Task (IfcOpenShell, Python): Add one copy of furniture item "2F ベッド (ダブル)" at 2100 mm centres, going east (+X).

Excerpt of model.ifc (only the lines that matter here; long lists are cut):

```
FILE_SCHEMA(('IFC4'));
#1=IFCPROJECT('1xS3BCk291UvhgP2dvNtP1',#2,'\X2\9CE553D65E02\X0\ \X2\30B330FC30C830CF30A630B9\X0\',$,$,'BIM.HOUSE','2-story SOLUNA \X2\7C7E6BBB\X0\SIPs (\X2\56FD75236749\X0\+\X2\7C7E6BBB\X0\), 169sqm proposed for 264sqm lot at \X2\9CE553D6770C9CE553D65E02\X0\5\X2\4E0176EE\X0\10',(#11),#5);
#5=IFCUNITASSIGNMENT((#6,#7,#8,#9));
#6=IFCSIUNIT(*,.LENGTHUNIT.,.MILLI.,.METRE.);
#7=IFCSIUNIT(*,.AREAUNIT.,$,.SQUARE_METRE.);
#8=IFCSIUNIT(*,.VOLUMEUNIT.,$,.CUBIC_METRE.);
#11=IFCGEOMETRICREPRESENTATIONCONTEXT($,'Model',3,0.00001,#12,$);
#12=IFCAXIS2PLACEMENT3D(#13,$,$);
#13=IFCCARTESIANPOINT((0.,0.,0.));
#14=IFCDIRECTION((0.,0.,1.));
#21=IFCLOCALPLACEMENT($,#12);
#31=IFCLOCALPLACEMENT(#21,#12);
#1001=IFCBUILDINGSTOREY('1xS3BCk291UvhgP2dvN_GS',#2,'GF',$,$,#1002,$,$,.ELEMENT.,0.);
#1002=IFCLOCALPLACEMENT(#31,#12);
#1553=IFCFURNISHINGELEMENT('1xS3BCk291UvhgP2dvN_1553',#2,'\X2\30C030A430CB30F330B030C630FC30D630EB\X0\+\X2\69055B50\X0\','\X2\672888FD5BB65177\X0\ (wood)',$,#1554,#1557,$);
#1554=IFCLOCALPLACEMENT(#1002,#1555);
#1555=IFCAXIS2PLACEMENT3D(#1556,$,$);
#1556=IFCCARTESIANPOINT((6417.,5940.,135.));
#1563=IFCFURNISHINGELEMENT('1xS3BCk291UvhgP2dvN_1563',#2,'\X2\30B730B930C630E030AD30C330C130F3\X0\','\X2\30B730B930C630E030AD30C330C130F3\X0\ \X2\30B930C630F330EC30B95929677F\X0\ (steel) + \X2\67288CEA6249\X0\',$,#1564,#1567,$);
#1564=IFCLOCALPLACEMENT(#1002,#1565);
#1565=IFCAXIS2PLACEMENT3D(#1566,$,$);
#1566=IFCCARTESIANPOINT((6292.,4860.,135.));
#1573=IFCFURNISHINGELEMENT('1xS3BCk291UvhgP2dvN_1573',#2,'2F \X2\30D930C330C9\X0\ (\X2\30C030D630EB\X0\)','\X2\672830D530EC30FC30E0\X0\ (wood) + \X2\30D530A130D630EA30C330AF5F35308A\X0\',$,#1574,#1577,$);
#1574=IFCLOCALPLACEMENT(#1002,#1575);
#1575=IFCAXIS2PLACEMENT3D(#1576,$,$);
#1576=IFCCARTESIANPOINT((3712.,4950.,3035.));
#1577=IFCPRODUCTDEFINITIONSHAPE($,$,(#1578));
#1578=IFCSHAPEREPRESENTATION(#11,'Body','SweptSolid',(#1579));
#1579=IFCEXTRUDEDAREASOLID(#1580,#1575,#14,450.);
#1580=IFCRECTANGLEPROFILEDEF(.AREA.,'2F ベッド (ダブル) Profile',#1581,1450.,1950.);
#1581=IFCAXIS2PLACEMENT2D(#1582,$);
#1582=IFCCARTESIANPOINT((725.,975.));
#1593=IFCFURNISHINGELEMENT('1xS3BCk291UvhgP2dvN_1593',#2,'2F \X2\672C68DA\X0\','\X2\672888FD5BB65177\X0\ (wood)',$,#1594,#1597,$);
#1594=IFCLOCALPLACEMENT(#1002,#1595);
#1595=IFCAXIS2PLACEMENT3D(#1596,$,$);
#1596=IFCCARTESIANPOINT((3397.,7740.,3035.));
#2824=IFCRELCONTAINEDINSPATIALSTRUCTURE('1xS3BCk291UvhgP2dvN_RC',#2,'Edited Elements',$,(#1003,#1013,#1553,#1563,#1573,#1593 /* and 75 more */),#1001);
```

```python
import numpy as np
import ifcopenshell
import ifcopenshell.api.geometry
import ifcopenshell.api.root
import ifcopenshell.util.element
import ifcopenshell.util.placement
import ifcopenshell.util.unit

model = ifcopenshell.open("model.ifc")
unit_scale = ifcopenshell.util.unit.calculate_unit_scale(model)


def reuse_history(source, copy):
    """copy_class also copies each property set's owner history, people and application; keep the originals."""
    for rel in copy.IsDefinedBy:
        if rel.is_a("IfcRelDefinesByProperties") and (history := rel.RelatingPropertyDefinition.OwnerHistory):
            rel.RelatingPropertyDefinition.OwnerHistory = source.OwnerHistory
            ifcopenshell.util.element.remove_deep2(model, history)


source = model.by_id(1573)
base = ifcopenshell.util.placement.get_local_placement(source.ObjectPlacement)
step = np.array([1.0, 0.0, 0.0]) * 2.1 / unit_scale

for i in range(1, 2):
    copy = ifcopenshell.api.root.copy_class(model, product=source)
    copy.Representation = ifcopenshell.util.element.copy_deep(
        model, source.Representation, exclude=["IfcGeometricRepresentationContext", "IfcRepresentationMap"]
    )
    reuse_history(source, copy)
    matrix = base.copy()
    matrix[:3, 3] += i * step
    print("added at", matrix[:3, 3].round(3) + 0.0)
    ifcopenshell.api.geometry.edit_object_placement(model, product=copy, matrix=matrix, is_si=False)

model.write("model_updated.ifc")
```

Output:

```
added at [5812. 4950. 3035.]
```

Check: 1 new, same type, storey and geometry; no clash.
